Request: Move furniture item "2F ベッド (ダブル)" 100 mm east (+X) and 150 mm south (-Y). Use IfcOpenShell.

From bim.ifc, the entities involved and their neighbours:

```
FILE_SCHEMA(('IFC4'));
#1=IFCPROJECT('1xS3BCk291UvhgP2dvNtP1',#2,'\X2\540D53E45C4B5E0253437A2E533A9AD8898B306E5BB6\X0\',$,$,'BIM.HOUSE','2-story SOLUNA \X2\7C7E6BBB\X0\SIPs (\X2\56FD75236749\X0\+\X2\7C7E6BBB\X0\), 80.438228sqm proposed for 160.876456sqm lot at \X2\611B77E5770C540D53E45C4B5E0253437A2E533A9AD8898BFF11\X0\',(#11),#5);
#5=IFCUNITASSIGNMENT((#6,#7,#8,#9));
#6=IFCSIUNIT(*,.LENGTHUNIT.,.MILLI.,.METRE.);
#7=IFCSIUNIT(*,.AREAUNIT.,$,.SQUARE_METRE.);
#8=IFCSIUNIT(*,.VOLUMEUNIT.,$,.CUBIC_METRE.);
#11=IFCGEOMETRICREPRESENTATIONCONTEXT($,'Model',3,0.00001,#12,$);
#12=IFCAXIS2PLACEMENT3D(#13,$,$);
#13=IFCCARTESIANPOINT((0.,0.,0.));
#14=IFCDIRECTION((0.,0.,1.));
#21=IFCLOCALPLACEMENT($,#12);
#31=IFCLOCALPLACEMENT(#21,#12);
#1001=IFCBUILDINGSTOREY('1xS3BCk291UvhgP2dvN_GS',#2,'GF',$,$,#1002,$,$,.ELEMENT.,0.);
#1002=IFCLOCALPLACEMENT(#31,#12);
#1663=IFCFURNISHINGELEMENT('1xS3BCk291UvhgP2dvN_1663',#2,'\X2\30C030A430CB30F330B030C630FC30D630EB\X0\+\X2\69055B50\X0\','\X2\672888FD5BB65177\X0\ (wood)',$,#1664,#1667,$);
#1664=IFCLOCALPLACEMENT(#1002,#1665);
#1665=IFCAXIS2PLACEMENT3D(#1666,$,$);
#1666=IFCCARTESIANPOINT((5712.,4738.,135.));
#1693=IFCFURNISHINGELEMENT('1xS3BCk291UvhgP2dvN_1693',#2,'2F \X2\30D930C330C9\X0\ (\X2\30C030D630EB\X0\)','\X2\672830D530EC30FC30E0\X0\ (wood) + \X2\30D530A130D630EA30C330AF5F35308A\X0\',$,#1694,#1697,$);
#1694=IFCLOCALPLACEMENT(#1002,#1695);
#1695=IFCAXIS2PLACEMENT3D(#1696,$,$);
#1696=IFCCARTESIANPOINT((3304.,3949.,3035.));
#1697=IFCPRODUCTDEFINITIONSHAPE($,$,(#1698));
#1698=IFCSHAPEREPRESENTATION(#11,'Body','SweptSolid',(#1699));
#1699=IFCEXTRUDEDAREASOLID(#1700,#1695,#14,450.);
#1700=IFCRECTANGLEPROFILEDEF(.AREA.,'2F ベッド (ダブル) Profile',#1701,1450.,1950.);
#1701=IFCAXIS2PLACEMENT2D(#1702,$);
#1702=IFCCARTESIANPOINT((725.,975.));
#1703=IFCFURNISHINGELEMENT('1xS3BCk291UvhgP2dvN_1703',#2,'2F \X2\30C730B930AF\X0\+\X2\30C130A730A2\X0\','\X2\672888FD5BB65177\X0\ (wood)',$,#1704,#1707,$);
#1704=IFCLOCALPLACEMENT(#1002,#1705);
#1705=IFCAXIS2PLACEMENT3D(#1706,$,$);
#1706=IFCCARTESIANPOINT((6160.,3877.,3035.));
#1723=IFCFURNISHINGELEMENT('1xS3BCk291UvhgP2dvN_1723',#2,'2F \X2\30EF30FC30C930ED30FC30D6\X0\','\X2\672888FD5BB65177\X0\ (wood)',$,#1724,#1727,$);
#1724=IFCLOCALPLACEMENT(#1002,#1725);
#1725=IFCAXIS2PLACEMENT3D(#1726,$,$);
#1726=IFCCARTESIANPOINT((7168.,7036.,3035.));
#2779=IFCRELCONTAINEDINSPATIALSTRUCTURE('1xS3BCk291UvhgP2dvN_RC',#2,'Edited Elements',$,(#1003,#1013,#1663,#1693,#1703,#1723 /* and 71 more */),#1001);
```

```python
import ifcopenshell
import ifcopenshell.api.geometry
import ifcopenshell.util.placement
import ifcopenshell.util.unit

model = ifcopenshell.open("bim.ifc")
unit_scale = ifcopenshell.util.unit.calculate_unit_scale(model)

item = model.by_id(1693)
matrix = ifcopenshell.util.placement.get_local_placement(item.ObjectPlacement)
matrix[0, 3] += 0.1 / unit_scale
matrix[1, 3] -= 0.15 / unit_scale
ifcopenshell.api.geometry.edit_object_placement(model, product=item, matrix=matrix, is_si=False)

print(ifcopenshell.util.placement.get_local_placement(item.ObjectPlacement).round(3) + 0.0)

model.write("bim-out.ifc")
```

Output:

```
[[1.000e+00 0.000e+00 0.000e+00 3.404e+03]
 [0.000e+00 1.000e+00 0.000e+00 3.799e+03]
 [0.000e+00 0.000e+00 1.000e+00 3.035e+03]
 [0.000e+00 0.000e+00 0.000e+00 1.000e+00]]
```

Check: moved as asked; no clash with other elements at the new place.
